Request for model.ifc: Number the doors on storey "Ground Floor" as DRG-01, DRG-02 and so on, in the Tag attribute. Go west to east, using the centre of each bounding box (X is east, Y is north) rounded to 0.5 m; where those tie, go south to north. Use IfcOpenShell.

First a look at what the model holds.

```python
import ifcopenshell
import ifcopenshell.util.element
import ifcopenshell.util.placement

model = ifcopenshell.open("model.ifc")
print(model.schema)
storey = next(s for s in model.by_type("IfcBuildingStorey") if s.Name == "Ground Floor")
doors = [e for e in ifcopenshell.util.element.get_decomposition(storey) if e.is_a("IfcDoor")]
for e in sorted(doors, key=lambda e: e.id()):
    origin = ifcopenshell.util.placement.get_local_placement(e.ObjectPlacement)[:3, 3]
    print(e.id(), e.Tag, e.Name, origin.round(2) + 0.0, sep=" | ")
```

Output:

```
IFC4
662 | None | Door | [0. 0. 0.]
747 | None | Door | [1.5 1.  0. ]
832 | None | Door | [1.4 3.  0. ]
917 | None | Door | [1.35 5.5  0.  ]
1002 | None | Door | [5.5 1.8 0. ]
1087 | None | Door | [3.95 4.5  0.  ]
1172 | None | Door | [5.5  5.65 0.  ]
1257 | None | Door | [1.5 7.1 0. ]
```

```python
import ifcopenshell
import ifcopenshell.geom
import ifcopenshell.util.element
import ifcopenshell.util.shape

model = ifcopenshell.open("model.ifc")
settings = ifcopenshell.geom.settings()
settings.set("use-world-coords", True)


def centre(element):
    shape = ifcopenshell.geom.create_shape(settings, element)
    return ifcopenshell.util.shape.get_bbox_centroid(shape.geometry)


storey = next(s for s in model.by_type("IfcBuildingStorey") if s.Name == "Ground Floor")
doors = [e for e in ifcopenshell.util.element.get_decomposition(storey) if e.is_a("IfcDoor")]

# Insertion points can sit at a corner or the storey origin, so sort by the geometry (in metres).
centres = {e: centre(e) for e in doors}
doors.sort(key=lambda e: (round(centres[e][0] / 0.5), centres[e][1]))

for i, e in enumerate(doors, start=1):
    number = f"DRG-{i:02d}"
    e.Tag = number
    print(e.id(), number)

model.write("model_rev.ifc")
```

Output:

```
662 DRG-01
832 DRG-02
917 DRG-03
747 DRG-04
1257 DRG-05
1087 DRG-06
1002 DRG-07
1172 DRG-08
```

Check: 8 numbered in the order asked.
